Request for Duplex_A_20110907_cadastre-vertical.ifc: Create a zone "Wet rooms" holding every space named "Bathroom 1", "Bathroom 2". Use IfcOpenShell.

First a look at what the model holds.

```python
import ifcopenshell

model = ifcopenshell.open("Duplex_A_20110907_cadastre-vertical.ifc")
print(model.schema)
seen = {}
for space in model.by_type("IfcSpace"):
    seen[space.LongName] = seen.get(space.LongName, 0) + 1
for name, count in sorted(seen.items(), key=str):
    print(count, "x", name)
print("zones:", [z.Name for z in model.by_type("IfcZone")][:20])
```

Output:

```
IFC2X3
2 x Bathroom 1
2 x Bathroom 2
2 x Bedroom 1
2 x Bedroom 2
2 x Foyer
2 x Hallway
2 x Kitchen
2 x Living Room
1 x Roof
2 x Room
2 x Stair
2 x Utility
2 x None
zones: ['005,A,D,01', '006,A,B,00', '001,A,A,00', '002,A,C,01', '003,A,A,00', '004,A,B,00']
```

```python
import ifcopenshell
import ifcopenshell.api.group
import ifcopenshell.api.root

model = ifcopenshell.open("Duplex_A_20110907_cadastre-vertical.ifc")

names = {"Bathroom 1", "Bathroom 2"}
spaces = [s for s in model.by_type("IfcSpace") if s.LongName in names]

zone = ifcopenshell.api.root.create_entity(model, ifc_class="IfcZone", name="Wet rooms")
ifcopenshell.api.group.assign_group(model, products=spaces, group=zone)
print(len(spaces), "spaces in", zone.Name)

model.write("Duplex_A_20110907_cadastre-vertical_edited.ifc")
```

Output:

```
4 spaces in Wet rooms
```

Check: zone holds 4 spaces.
